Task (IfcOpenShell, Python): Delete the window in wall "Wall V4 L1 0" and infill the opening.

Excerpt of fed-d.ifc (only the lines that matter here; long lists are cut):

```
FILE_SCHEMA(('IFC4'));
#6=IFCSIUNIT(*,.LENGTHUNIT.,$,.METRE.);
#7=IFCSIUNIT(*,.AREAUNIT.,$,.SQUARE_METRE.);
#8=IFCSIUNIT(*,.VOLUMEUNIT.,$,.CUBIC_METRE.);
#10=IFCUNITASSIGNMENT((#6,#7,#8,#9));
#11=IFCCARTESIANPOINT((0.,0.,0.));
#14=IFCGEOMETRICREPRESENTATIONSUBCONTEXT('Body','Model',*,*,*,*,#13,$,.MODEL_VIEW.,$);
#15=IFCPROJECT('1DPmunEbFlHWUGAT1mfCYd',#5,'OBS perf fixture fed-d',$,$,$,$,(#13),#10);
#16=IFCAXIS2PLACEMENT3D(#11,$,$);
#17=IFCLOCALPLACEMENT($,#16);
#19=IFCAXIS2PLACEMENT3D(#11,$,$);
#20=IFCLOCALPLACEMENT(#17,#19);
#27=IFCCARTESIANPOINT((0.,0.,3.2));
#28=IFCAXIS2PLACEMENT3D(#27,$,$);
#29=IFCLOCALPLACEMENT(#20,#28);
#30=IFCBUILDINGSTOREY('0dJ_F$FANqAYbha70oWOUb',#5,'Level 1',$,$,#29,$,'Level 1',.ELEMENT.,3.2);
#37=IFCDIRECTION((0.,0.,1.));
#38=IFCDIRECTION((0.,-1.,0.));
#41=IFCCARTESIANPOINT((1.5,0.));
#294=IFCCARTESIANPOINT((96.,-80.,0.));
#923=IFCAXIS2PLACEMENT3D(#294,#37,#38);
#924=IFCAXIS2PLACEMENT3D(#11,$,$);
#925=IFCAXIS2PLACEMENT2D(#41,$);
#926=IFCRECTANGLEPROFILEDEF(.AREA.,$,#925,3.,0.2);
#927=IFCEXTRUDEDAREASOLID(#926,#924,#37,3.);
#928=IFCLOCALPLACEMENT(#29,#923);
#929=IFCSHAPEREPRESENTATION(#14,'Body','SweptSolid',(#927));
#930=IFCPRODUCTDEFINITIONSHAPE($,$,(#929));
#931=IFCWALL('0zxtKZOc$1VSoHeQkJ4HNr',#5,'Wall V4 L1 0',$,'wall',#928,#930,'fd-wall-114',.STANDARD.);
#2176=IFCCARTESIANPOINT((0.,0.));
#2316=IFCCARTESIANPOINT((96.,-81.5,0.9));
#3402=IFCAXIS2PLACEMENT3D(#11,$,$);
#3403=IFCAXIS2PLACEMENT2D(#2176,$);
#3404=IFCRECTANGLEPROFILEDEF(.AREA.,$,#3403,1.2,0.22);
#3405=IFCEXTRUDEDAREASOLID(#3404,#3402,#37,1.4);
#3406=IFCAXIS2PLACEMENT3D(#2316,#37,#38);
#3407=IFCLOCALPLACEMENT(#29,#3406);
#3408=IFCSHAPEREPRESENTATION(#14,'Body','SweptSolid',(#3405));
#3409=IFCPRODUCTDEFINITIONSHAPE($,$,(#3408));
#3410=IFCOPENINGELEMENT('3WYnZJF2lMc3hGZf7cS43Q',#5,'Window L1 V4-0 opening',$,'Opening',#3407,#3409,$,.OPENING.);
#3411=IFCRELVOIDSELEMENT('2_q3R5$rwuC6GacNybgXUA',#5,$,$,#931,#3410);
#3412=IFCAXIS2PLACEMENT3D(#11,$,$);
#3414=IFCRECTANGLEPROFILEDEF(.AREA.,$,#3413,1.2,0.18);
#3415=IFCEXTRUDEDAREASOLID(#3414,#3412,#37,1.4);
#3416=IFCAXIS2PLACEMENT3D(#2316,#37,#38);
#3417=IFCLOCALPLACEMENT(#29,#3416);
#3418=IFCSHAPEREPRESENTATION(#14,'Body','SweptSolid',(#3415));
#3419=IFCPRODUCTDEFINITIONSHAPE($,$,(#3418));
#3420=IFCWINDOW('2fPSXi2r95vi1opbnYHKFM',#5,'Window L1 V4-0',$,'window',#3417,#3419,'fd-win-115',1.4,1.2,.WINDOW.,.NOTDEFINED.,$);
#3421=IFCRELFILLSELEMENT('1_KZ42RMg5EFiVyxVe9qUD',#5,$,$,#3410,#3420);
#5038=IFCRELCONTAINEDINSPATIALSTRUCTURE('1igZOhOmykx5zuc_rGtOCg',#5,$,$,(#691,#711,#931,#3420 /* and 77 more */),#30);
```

```python
import ifcopenshell
import ifcopenshell.api.feature
import ifcopenshell.api.root
import ifcopenshell.geom
import ifcopenshell.util.shape

model = ifcopenshell.open("fed-d.ifc")
settings = ifcopenshell.geom.settings()


def volume(element):
    """Net volume in cubic metres, openings subtracted."""
    shape = ifcopenshell.geom.create_shape(settings, element)
    return ifcopenshell.util.shape.get_volume(shape.geometry)


window = model.by_guid("2fPSXi2r95vi1opbnYHKFM")
opening = window.FillsVoids[0].RelatingOpeningElement
wall = opening.VoidsElements[0].RelatingBuildingElement
before = volume(wall)

ifcopenshell.api.root.remove_product(model, product=window)
ifcopenshell.api.feature.remove_feature(model, feature=opening)

after = volume(wall)

print(f"wall volume {before:.3f} -> {after:.3f} m3")

model.write("fed-d_updated.ifc")
```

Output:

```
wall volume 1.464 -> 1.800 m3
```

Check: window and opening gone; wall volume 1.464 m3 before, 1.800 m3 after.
